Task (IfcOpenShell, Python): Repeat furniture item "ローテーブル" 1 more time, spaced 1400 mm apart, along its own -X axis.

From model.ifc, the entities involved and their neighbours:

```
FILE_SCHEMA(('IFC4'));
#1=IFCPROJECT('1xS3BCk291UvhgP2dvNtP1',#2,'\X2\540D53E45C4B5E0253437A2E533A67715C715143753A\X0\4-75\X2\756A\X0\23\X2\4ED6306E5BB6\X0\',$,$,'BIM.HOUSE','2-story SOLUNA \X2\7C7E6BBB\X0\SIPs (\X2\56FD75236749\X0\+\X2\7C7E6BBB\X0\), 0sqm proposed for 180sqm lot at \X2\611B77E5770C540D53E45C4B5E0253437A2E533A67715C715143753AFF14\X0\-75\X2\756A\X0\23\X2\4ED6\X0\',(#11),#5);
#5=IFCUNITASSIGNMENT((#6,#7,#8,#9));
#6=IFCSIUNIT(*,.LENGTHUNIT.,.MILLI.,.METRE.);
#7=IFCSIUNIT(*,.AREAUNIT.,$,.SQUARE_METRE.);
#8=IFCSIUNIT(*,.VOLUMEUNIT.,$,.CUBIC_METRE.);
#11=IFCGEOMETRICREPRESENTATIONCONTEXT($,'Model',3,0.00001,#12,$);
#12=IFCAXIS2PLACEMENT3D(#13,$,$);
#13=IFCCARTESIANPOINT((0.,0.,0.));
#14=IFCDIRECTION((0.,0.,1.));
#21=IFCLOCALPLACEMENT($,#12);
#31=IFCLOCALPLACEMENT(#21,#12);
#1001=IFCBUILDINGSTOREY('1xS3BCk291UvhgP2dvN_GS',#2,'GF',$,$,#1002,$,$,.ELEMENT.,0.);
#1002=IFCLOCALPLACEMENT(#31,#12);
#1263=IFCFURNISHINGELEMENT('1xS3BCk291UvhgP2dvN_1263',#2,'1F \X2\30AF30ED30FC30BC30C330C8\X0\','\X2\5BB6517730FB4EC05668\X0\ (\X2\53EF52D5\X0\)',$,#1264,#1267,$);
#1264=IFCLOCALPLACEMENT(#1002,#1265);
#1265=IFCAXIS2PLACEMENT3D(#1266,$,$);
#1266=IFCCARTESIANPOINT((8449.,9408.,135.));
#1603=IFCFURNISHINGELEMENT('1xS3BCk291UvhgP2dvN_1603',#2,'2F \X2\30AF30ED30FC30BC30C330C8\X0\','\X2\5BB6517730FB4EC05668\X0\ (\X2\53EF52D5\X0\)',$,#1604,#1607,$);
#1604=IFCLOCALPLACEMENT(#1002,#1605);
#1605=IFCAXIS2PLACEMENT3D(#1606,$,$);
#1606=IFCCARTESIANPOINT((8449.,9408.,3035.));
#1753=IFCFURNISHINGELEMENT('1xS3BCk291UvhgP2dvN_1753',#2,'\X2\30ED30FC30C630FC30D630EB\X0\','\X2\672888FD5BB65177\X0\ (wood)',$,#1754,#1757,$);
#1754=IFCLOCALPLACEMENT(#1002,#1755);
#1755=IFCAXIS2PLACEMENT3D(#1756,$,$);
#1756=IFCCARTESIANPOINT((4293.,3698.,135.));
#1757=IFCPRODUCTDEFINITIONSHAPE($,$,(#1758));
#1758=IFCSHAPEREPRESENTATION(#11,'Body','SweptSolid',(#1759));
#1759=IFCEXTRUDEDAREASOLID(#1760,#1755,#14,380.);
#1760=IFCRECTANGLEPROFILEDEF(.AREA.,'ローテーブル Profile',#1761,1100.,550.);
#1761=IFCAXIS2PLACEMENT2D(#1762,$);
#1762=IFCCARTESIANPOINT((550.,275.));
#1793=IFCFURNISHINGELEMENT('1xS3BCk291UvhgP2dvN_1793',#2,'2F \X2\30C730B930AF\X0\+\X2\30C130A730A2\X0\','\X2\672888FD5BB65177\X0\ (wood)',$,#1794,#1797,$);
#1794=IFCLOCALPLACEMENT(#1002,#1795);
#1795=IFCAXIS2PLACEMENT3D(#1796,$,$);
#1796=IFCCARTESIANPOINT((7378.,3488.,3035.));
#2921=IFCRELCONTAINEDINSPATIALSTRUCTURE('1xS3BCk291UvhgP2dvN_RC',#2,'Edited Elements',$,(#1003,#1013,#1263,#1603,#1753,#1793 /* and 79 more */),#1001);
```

```python
import ifcopenshell
import ifcopenshell.api.geometry
import ifcopenshell.api.root
import ifcopenshell.util.element
import ifcopenshell.util.placement
import ifcopenshell.util.unit

model = ifcopenshell.open("model.ifc")
unit_scale = ifcopenshell.util.unit.calculate_unit_scale(model)


def reuse_history(source, copy):
    """copy_class also copies each property set's owner history, people and application; keep the originals."""
    for rel in copy.IsDefinedBy:
        if rel.is_a("IfcRelDefinesByProperties") and (history := rel.RelatingPropertyDefinition.OwnerHistory):
            rel.RelatingPropertyDefinition.OwnerHistory = source.OwnerHistory
            ifcopenshell.util.element.remove_deep2(model, history)


source = model.by_guid("1xS3BCk291UvhgP2dvN_1753")
base = ifcopenshell.util.placement.get_local_placement(source.ObjectPlacement)
step = -base[:3, 0] * 1.4 / unit_scale

for i in range(1, 2):
    copy = ifcopenshell.api.root.copy_class(model, product=source)
    copy.Representation = ifcopenshell.util.element.copy_deep(
        model, source.Representation, exclude=["IfcGeometricRepresentationContext", "IfcRepresentationMap"]
    )
    reuse_history(source, copy)
    matrix = base.copy()
    matrix[:3, 3] += i * step
    print("added at", matrix[:3, 3].round(3) + 0.0)
    ifcopenshell.api.geometry.edit_object_placement(model, product=copy, matrix=matrix, is_si=False)

model.write("model_updated.ifc")
```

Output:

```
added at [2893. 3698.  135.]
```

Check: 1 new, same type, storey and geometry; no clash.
